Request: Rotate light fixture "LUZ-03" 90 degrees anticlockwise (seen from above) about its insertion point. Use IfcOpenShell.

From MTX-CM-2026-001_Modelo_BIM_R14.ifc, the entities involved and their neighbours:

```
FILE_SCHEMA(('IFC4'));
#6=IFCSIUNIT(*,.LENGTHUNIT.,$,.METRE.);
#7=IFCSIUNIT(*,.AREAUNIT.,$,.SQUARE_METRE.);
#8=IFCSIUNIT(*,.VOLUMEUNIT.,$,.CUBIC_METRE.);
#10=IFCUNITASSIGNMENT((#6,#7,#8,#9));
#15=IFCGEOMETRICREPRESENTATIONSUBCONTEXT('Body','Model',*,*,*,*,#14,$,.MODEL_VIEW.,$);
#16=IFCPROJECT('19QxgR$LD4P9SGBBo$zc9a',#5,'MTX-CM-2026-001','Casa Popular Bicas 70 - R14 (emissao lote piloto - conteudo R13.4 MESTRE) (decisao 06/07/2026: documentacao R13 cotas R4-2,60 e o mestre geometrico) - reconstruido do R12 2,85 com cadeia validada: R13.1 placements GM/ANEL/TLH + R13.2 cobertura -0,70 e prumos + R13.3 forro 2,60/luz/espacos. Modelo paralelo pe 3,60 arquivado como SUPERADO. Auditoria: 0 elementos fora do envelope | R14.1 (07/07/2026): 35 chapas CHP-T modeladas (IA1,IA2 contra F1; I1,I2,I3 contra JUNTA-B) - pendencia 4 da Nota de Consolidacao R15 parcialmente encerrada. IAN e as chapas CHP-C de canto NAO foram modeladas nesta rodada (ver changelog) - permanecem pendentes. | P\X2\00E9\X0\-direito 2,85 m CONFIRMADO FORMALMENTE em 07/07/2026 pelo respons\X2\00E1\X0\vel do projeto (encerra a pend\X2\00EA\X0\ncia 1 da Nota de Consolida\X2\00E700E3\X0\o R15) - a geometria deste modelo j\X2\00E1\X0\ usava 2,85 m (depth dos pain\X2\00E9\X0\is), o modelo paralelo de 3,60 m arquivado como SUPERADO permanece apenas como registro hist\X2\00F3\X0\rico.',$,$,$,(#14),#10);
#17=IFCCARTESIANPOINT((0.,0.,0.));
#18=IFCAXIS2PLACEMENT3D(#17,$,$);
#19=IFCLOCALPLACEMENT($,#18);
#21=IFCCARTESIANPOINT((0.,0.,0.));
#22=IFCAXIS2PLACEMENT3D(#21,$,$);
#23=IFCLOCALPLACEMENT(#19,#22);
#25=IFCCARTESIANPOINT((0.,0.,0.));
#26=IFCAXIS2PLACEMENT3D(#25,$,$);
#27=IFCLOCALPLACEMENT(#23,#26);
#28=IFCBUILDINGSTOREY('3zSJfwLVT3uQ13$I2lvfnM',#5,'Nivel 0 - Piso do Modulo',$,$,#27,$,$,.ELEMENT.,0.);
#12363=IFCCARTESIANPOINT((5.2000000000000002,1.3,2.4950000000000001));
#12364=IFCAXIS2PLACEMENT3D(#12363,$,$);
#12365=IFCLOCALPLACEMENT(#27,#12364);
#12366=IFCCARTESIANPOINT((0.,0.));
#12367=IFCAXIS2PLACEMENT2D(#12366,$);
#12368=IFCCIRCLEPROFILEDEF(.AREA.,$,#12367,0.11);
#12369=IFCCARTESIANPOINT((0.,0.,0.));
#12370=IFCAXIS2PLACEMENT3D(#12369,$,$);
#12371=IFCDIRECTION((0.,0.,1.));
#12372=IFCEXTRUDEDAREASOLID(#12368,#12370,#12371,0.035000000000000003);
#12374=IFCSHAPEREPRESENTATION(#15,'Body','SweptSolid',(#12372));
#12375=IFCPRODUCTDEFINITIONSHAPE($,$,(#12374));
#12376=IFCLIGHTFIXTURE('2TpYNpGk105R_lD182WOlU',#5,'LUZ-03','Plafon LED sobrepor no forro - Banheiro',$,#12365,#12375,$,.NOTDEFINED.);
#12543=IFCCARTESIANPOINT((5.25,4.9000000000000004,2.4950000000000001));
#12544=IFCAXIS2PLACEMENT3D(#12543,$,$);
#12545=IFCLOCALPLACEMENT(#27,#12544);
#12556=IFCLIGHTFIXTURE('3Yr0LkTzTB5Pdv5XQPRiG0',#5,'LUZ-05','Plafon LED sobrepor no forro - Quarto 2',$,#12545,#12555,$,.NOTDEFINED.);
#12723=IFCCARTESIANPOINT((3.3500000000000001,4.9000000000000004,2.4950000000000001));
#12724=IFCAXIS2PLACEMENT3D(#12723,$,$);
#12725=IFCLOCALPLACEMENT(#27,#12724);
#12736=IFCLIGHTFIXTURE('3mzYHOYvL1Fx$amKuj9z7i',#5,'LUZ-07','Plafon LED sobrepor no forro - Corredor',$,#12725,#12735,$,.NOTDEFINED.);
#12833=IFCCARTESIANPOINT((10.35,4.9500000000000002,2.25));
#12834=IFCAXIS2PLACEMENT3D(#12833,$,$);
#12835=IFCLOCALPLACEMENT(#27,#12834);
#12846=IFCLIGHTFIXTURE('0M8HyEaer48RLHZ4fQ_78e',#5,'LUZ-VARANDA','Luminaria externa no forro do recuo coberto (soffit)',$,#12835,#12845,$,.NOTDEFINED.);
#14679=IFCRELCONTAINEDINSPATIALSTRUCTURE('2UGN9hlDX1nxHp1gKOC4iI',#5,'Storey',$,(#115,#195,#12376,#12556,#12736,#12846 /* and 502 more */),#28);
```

```python
import ifcopenshell
import ifcopenshell.api.geometry
import ifcopenshell.util.placement

model = ifcopenshell.open("MTX-CM-2026-001_Modelo_BIM_R14.ifc")

item = model.by_guid("2TpYNpGk105R_lD182WOlU")
matrix = ifcopenshell.util.placement.get_local_placement(item.ObjectPlacement)
matrix = matrix @ ifcopenshell.util.placement.rotation(90, "Z")
ifcopenshell.api.geometry.edit_object_placement(model, product=item, matrix=matrix, is_si=False)

print(ifcopenshell.util.placement.get_local_placement(item.ObjectPlacement).round(3) + 0.0)

model.write("MTX-CM-2026-001_Modelo_BIM_R14_updated.ifc")
```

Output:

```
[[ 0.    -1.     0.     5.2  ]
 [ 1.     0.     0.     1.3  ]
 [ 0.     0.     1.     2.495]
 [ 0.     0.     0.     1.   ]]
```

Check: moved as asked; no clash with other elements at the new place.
